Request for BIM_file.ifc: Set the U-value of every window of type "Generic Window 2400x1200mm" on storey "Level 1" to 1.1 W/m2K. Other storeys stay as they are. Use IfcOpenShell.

First a look at what the model holds.

```python
import ifcopenshell
import ifcopenshell.util.element

model = ifcopenshell.open("BIM_file.ifc")
print(model.schema)
storey = next(s for s in model.by_type("IfcBuildingStorey") if s.Name == "Level 1")
windows = [e for e in ifcopenshell.util.element.get_decomposition(storey) if e.is_a("IfcWindow")]
seen = {}
for e in windows:
    element_type = ifcopenshell.util.element.get_type(e)
    key = (element_type.Name if element_type != e and element_type else None, ifcopenshell.util.element.get_pset(e, "Pset_WindowCommon", "ThermalTransmittance"))
    seen[key] = seen.get(key, 0) + 1
for (name, value), count in sorted(seen.items(), key=str):
    print(count, "x", name, "|", value)
```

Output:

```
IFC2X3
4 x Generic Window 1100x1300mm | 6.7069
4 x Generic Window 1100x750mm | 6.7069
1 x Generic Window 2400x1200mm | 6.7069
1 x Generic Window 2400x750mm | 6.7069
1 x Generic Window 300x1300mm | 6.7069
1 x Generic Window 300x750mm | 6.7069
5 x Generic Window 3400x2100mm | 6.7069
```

```python
import ifcopenshell
import ifcopenshell.api.pset
import ifcopenshell.util.element

model = ifcopenshell.open("BIM_file.ifc")

storey = next(s for s in model.by_type("IfcBuildingStorey") if s.Name == "Level 1")
windows = [e for e in ifcopenshell.util.element.get_decomposition(storey) if e.is_a("IfcWindow")]

count = 0
for e in windows:
    element_type = ifcopenshell.util.element.get_type(e)
    if element_type in (None, e) or element_type.Name != "Generic Window 2400x1200mm":
        continue
    # add_pset returns the element's existing set when there is one.
    pset = ifcopenshell.api.pset.add_pset(model, product=e, name="Pset_WindowCommon")
    ifcopenshell.api.pset.edit_pset(model, pset=pset, properties={"ThermalTransmittance": 1.1})
    count += 1

print(count, "windows updated")

model.write("BIM_file_v2.ifc")
```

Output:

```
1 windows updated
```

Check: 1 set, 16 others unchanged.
